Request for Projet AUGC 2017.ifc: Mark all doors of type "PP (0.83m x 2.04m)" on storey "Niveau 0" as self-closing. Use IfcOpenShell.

First a look at what the model holds.

```python
import ifcopenshell
import ifcopenshell.util.element

model = ifcopenshell.open("Projet AUGC 2017.ifc")
print(model.schema)
storey = next(s for s in model.by_type("IfcBuildingStorey") if s.Name == "Niveau 0")
doors = [e for e in ifcopenshell.util.element.get_decomposition(storey) if e.is_a("IfcDoor")]
seen = {}
for e in doors:
    element_type = ifcopenshell.util.element.get_type(e)
    key = (element_type.Name if element_type != e and element_type else None, ifcopenshell.util.element.get_pset(e, "Pset_DoorCommon", "SelfClosing"))
    seen[key] = seen.get(key, 0) + 1
for (name, value), count in sorted(seen.items(), key=str):
    print(count, "x", name, "|", value)
```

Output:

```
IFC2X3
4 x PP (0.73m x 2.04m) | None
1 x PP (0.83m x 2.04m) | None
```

```python
import ifcopenshell
import ifcopenshell.api.pset
import ifcopenshell.util.element

model = ifcopenshell.open("Projet AUGC 2017.ifc")

storey = next(s for s in model.by_type("IfcBuildingStorey") if s.Name == "Niveau 0")
doors = [e for e in ifcopenshell.util.element.get_decomposition(storey) if e.is_a("IfcDoor")]

count = 0
for e in doors:
    element_type = ifcopenshell.util.element.get_type(e)
    if element_type in (None, e) or element_type.Name != "PP (0.83m x 2.04m)":
        continue
    # add_pset returns the element's existing set when there is one.
    pset = ifcopenshell.api.pset.add_pset(model, product=e, name="Pset_DoorCommon")
    ifcopenshell.api.pset.edit_pset(model, pset=pset, properties={"SelfClosing": True})
    count += 1

print(count, "doors updated")

model.write("Projet AUGC 2017_edited.ifc")
```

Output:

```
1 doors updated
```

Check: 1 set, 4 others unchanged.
